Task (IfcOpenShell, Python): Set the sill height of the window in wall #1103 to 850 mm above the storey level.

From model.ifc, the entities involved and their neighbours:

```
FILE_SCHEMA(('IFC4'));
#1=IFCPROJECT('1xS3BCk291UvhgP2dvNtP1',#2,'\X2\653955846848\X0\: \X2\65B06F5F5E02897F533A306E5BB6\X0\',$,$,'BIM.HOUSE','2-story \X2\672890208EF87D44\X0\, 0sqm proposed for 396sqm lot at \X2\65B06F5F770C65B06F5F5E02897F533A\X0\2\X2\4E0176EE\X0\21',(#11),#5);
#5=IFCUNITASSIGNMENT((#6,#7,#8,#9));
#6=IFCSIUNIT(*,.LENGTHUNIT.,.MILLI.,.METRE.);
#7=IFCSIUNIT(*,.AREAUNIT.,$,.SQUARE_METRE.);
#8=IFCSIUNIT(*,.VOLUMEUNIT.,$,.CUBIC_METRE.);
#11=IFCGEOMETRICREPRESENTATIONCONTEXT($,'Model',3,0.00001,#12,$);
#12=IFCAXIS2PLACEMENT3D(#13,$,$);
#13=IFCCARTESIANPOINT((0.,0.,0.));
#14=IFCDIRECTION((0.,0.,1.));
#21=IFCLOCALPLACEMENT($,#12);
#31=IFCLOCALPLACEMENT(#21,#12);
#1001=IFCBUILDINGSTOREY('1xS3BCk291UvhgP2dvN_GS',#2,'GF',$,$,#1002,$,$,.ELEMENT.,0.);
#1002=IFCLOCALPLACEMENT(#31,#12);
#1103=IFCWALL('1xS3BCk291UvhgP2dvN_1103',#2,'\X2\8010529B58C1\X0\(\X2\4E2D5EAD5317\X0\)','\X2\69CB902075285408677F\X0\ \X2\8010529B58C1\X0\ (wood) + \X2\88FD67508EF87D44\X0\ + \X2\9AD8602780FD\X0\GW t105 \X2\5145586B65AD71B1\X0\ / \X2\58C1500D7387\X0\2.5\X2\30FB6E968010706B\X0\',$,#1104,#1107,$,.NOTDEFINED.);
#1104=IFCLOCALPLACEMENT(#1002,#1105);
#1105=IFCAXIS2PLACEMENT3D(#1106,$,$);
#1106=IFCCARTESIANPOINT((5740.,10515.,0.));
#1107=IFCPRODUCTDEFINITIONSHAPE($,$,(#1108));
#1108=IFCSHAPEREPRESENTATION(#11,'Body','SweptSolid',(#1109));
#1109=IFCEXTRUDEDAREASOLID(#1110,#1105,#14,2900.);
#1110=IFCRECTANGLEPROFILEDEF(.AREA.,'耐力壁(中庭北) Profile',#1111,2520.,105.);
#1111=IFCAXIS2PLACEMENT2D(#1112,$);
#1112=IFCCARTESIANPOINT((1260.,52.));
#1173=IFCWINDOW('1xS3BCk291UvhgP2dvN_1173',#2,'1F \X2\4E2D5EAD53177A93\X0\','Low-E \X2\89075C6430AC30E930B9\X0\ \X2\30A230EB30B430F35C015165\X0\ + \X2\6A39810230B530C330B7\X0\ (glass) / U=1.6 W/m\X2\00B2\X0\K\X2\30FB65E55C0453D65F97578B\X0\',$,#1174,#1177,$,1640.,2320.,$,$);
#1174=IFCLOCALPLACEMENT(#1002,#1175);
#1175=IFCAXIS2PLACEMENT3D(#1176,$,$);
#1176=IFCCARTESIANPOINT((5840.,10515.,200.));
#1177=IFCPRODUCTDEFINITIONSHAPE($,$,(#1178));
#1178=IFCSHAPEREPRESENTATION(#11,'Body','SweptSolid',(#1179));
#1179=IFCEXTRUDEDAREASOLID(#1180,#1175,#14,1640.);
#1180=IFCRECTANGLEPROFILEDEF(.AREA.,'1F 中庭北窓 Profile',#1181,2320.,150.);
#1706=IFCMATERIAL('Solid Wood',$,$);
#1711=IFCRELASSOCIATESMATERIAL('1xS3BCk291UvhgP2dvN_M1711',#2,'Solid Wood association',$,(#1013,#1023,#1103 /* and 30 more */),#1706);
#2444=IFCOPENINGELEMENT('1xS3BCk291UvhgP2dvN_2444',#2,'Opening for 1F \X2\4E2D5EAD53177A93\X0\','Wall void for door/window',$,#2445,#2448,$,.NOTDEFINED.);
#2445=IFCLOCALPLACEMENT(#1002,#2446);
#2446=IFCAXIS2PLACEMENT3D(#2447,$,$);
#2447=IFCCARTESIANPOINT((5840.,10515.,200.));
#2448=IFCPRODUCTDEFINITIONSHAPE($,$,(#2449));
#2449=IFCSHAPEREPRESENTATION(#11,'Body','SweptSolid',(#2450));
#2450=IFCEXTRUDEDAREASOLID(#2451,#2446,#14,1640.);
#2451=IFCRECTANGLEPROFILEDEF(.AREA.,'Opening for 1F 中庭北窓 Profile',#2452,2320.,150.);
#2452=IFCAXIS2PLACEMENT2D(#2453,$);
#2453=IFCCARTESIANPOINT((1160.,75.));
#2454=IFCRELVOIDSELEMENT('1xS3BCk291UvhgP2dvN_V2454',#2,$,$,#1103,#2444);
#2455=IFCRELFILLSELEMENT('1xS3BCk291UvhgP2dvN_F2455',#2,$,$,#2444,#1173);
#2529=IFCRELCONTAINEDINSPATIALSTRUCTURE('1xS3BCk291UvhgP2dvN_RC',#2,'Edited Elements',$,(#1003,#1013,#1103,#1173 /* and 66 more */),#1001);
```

```python
import numpy as np
import ifcopenshell
import ifcopenshell.api.geometry
import ifcopenshell.geom
import ifcopenshell.util.element
import ifcopenshell.util.placement
import ifcopenshell.util.shape
import ifcopenshell.util.unit

model = ifcopenshell.open("model.ifc")
unit_scale = ifcopenshell.util.unit.calculate_unit_scale(model)

window = model.by_id(1173)
opening = window.FillsVoids[0].RelatingOpeningElement
storey = ifcopenshell.util.element.get_container(window, ifc_class="IfcBuildingStorey")
level = ifcopenshell.util.placement.get_local_placement(storey.ObjectPlacement)[2, 3]

# The opening's origin need not be at the sill, so measure its lowest point.
shape = ifcopenshell.geom.create_shape(ifcopenshell.geom.settings(), opening)
bottom = ifcopenshell.util.shape.get_shape_bottom_elevation(shape, shape.geometry) / unit_scale
dz = level + 850.0 - bottom

shift = np.array([0.0, 0.0, dz])
# The window is not placed relative to its opening, so move both.
for product in (opening, window):
    matrix = ifcopenshell.util.placement.get_local_placement(product.ObjectPlacement)
    matrix[:3, 3] += shift
    ifcopenshell.api.geometry.edit_object_placement(model, product=product, matrix=matrix, is_si=False)

print(f"moved by {dz * unit_scale:+.3f} m")

model.write("model_rev.ifc")
```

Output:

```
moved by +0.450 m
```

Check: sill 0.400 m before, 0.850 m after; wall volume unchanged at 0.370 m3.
